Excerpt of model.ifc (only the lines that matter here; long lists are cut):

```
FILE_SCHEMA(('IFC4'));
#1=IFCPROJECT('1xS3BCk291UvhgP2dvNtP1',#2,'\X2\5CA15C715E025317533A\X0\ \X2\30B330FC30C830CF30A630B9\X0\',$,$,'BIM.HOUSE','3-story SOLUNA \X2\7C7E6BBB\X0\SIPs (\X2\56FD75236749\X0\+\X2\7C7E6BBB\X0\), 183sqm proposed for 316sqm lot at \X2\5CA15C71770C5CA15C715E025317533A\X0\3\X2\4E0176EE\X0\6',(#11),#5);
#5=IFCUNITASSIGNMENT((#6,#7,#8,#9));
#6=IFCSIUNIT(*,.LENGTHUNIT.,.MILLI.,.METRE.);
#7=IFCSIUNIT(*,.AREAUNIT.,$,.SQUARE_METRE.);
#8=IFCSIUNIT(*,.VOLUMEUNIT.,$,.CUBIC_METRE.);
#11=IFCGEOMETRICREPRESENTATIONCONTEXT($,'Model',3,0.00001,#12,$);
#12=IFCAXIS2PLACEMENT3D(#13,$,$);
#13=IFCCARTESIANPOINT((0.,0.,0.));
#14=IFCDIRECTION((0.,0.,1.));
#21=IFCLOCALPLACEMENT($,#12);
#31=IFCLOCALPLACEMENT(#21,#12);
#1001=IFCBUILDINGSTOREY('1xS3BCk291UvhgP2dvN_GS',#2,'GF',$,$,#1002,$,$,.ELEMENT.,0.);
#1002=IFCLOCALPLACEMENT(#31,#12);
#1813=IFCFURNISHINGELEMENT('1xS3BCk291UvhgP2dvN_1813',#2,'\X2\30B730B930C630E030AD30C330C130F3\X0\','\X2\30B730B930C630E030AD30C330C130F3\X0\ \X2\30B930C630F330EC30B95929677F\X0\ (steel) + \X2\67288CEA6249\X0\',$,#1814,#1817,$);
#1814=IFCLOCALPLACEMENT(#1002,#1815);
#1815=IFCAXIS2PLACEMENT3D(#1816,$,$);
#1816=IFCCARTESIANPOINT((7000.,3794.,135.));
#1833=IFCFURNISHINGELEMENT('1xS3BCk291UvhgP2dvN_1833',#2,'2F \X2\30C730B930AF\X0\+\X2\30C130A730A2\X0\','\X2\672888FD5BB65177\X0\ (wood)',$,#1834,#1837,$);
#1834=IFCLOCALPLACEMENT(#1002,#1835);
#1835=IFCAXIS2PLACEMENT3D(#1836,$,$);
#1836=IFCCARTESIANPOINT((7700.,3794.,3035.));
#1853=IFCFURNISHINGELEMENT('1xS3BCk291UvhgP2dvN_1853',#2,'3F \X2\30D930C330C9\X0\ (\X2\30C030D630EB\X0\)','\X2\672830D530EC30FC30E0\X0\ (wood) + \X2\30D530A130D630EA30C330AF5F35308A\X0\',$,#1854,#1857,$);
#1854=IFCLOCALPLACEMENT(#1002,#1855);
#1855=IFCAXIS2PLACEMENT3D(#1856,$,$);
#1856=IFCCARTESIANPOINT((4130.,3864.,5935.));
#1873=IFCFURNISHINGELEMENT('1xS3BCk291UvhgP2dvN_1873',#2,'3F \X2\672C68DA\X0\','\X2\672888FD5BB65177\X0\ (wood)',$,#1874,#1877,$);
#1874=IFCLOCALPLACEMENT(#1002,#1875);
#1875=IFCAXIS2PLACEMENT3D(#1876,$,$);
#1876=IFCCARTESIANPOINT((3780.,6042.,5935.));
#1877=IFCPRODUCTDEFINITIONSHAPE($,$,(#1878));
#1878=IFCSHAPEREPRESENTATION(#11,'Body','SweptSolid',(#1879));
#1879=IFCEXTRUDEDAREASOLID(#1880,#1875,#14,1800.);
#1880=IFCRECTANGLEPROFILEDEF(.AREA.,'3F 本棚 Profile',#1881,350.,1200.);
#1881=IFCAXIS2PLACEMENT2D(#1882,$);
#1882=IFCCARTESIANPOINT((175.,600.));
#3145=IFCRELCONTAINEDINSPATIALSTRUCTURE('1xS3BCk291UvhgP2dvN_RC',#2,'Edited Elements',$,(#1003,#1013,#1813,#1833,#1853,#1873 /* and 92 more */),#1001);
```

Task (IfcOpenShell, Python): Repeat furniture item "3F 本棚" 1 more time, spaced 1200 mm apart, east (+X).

```python
import numpy as np
import ifcopenshell
import ifcopenshell.api.geometry
import ifcopenshell.api.root
import ifcopenshell.util.element
import ifcopenshell.util.placement
import ifcopenshell.util.unit

model = ifcopenshell.open("model.ifc")
unit_scale = ifcopenshell.util.unit.calculate_unit_scale(model)


def reuse_history(source, copy):
    """copy_class also copies each property set's owner history, people and application; keep the originals."""
    for rel in copy.IsDefinedBy:
        if rel.is_a("IfcRelDefinesByProperties") and (history := rel.RelatingPropertyDefinition.OwnerHistory):
            rel.RelatingPropertyDefinition.OwnerHistory = source.OwnerHistory
            ifcopenshell.util.element.remove_deep2(model, history)


source = model.by_guid("1xS3BCk291UvhgP2dvN_1873")
base = ifcopenshell.util.placement.get_local_placement(source.ObjectPlacement)
step = np.array([1.0, 0.0, 0.0]) * 1.2 / unit_scale

for i in range(1, 2):
    copy = ifcopenshell.api.root.copy_class(model, product=source)
    copy.Representation = ifcopenshell.util.element.copy_deep(
        model, source.Representation, exclude=["IfcGeometricRepresentationContext", "IfcRepresentationMap"]
    )
    reuse_history(source, copy)
    matrix = base.copy()
    matrix[:3, 3] += i * step
    print("added at", matrix[:3, 3].round(3) + 0.0)
    ifcopenshell.api.geometry.edit_object_placement(model, product=copy, matrix=matrix, is_si=False)

model.write("model-out.ifc")
```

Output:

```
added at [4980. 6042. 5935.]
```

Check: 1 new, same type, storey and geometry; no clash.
